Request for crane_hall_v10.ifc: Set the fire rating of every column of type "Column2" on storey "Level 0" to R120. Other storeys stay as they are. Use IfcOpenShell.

First a look at what the model holds.

```python
import ifcopenshell
import ifcopenshell.util.element

model = ifcopenshell.open("crane_hall_v10.ifc")
print(model.schema)
storey = next(s for s in model.by_type("IfcBuildingStorey") if s.Name == "Level 0")
columns = [e for e in ifcopenshell.util.element.get_decomposition(storey) if e.is_a("IfcColumn")]
seen = {}
for e in columns:
    element_type = ifcopenshell.util.element.get_type(e)
    key = (element_type.Name if element_type != e and element_type else None, ifcopenshell.util.element.get_pset(e, "Pset_ColumnCommon", "FireRating"))
    seen[key] = seen.get(key, 0) + 1
for (name, value), count in sorted(seen.items(), key=str):
    print(count, "x", name, "|", value)
```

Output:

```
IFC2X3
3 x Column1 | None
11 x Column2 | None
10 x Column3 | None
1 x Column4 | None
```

```python
import ifcopenshell
import ifcopenshell.api.pset
import ifcopenshell.util.element

model = ifcopenshell.open("crane_hall_v10.ifc")

storey = next(s for s in model.by_type("IfcBuildingStorey") if s.Name == "Level 0")
columns = [e for e in ifcopenshell.util.element.get_decomposition(storey) if e.is_a("IfcColumn")]

count = 0
for e in columns:
    element_type = ifcopenshell.util.element.get_type(e)
    if element_type in (None, e) or element_type.Name != "Column2":
        continue
    # add_pset returns the element's existing set when there is one.
    pset = ifcopenshell.api.pset.add_pset(model, product=e, name="Pset_ColumnCommon")
    ifcopenshell.api.pset.edit_pset(model, pset=pset, properties={"FireRating": "R120"})
    count += 1

print(count, "columns updated")

model.write("crane_hall_v10_edited.ifc")
```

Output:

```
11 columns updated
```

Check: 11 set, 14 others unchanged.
